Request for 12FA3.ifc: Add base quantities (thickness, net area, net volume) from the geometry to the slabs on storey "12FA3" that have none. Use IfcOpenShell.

First a look at what the model holds.

```python
import ifcopenshell
import ifcopenshell.util.element
import ifcopenshell.util.unit

model = ifcopenshell.open("12FA3.ifc")
print(model.schema)
for unit_type in ("LENGTHUNIT", "AREAUNIT", "VOLUMEUNIT"):
    print(unit_type, ifcopenshell.util.unit.calculate_unit_scale(model, unit_type))
storey = next(s for s in model.by_type("IfcBuildingStorey") if s.Name == "12FA3")
slabs = [e for e in ifcopenshell.util.element.get_decomposition(storey) if e.is_a("IfcSlab")]
for e in sorted(slabs, key=lambda e: e.id()):
    print(e.id(), e.is_a(), e.Name, list(ifcopenshell.util.element.get_psets(e, qtos_only=True)), sep=" | ")
```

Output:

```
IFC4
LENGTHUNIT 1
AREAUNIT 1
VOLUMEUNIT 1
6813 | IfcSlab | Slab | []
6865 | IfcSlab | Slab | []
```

```python
import ifcopenshell
import ifcopenshell.api.pset
import ifcopenshell.geom
import ifcopenshell.util.element
import ifcopenshell.util.shape
import ifcopenshell.util.unit

model = ifcopenshell.open("12FA3.ifc")
unit_scale = ifcopenshell.util.unit.calculate_unit_scale(model)
area_scale = ifcopenshell.util.unit.calculate_unit_scale(model, "AREAUNIT")
volume_scale = ifcopenshell.util.unit.calculate_unit_scale(model, "VOLUMEUNIT")
settings = ifcopenshell.geom.settings()

storey = next(s for s in model.by_type("IfcBuildingStorey") if s.Name == "12FA3")
slabs = [e for e in ifcopenshell.util.element.get_decomposition(storey) if e.is_a("IfcSlab")]

for e in sorted(slabs, key=lambda e: e.id()):
    if ifcopenshell.util.element.get_psets(e, qtos_only=True, should_inherit=False):
        continue
    # Geometry comes back in metres, in the element's own axes.
    shape = ifcopenshell.geom.create_shape(settings, e)
    values = {
        "Width": ifcopenshell.util.shape.get_z(shape.geometry) / unit_scale,
        "NetArea": ifcopenshell.util.shape.get_footprint_area(shape.geometry) / area_scale,
        "NetVolume": ifcopenshell.util.shape.get_volume(shape.geometry) / volume_scale,
    }
    qto = ifcopenshell.api.pset.add_qto(model, product=e, name="Qto_SlabBaseQuantities")
    ifcopenshell.api.pset.edit_qto(model, qto=qto, properties=values)
    print(e.id(), {k: round(v, 3) for k, v in values.items()})

model.write("12FA3_v2.ifc")
```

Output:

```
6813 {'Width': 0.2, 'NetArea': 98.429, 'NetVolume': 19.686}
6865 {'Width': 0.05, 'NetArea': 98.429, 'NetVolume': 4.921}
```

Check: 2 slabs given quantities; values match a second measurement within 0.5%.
